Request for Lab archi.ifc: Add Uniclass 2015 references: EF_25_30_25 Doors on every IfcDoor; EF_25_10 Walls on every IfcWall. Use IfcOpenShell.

First a look at what the model holds.

```python
import ifcopenshell

model = ifcopenshell.open("Lab archi.ifc")
print(model.schema)
print("classifications:", [c.Name for c in model.by_type("IfcClassification")])
for ifc_class in ("IfcDoor", "IfcRoof", "IfcStair", "IfcWall", "IfcWindow"):
    print(ifc_class, len(model.by_type(ifc_class)))
```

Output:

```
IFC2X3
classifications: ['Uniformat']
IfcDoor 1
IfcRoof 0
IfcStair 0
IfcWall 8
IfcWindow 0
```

```python
import ifcopenshell
import ifcopenshell.api.classification

model = ifcopenshell.open("Lab archi.ifc")

# IFC2X3 requires Source and Edition and has no link from the project to the system.
system = model.create_entity("IfcClassification", Source="NBS", Edition="2015", Name="Uniclass 2015")

codes = {
    "IfcDoor": ("EF_25_30_25", "Doors"),
    "IfcWall": ("EF_25_10", "Walls"),
}
for ifc_class, (code, name) in codes.items():
    products = model.by_type(ifc_class)
    ifcopenshell.api.classification.add_reference(
        model, products=products, classification=system, identification=code, name=name
    )
    print(code, len(products))

model.write("Lab archi_v2.ifc")
```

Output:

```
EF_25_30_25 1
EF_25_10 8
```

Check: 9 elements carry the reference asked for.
